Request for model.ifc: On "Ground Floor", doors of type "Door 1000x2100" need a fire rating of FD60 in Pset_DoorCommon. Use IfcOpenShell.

First a look at what the model holds.

```python
import ifcopenshell
import ifcopenshell.util.element

model = ifcopenshell.open("model.ifc")
print(model.schema)
storey = next(s for s in model.by_type("IfcBuildingStorey") if s.Name == "Ground Floor")
doors = [e for e in ifcopenshell.util.element.get_decomposition(storey) if e.is_a("IfcDoor")]
seen = {}
for e in doors:
    element_type = ifcopenshell.util.element.get_type(e)
    key = (element_type.Name if element_type != e and element_type else None, ifcopenshell.util.element.get_pset(e, "Pset_DoorCommon", "FireRating"))
    seen[key] = seen.get(key, 0) + 1
for (name, value), count in sorted(seen.items(), key=str):
    print(count, "x", name, "|", value)
```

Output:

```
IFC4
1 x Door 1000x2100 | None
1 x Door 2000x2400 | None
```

```python
import ifcopenshell
import ifcopenshell.api.pset
import ifcopenshell.util.element

model = ifcopenshell.open("model.ifc")

storey = next(s for s in model.by_type("IfcBuildingStorey") if s.Name == "Ground Floor")
doors = [e for e in ifcopenshell.util.element.get_decomposition(storey) if e.is_a("IfcDoor")]

count = 0
for e in doors:
    element_type = ifcopenshell.util.element.get_type(e)
    if element_type in (None, e) or element_type.Name != "Door 1000x2100":
        continue
    # add_pset returns the element's existing set when there is one.
    pset = ifcopenshell.api.pset.add_pset(model, product=e, name="Pset_DoorCommon")
    ifcopenshell.api.pset.edit_pset(model, pset=pset, properties={"FireRating": "FD60"})
    count += 1

print(count, "doors updated")

model.write("model_rev.ifc")
```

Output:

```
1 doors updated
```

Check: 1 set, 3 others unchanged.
